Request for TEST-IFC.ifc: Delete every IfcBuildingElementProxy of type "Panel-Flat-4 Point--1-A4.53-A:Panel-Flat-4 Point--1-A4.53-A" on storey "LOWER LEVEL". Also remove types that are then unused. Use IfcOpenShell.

First a look at what the model holds.

```python
import ifcopenshell
import ifcopenshell.util.element

model = ifcopenshell.open("TEST-IFC.ifc")
print(model.schema)
storey = next(s for s in model.by_type("IfcBuildingStorey") if s.Name == "LOWER LEVEL")
proxies = [e for e in ifcopenshell.util.element.get_decomposition(storey) if e.is_a("IfcBuildingElementProxy")]
seen = {}
for e in proxies:
    element_type = ifcopenshell.util.element.get_type(e)
    name = element_type.Name if element_type not in (None, e) else None
    seen[name] = seen.get(name, 0) + 1
for name, count in sorted(seen.items(), key=str):
    print(count, "x", name)
```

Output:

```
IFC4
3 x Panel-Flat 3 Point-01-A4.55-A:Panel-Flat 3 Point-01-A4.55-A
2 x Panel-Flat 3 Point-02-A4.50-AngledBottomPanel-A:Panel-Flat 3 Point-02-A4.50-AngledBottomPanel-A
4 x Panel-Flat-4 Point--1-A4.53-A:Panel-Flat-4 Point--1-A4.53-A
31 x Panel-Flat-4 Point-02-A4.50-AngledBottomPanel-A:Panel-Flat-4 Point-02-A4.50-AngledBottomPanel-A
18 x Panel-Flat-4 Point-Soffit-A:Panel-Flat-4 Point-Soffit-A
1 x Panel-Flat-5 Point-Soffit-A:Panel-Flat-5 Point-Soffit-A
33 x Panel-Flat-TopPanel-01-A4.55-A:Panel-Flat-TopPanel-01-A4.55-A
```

```python
import ifcopenshell
import ifcopenshell.api.root
import ifcopenshell.util.element

model = ifcopenshell.open("TEST-IFC.ifc")

storey = next(s for s in model.by_type("IfcBuildingStorey") if s.Name == "LOWER LEVEL")
proxies = [e for e in ifcopenshell.util.element.get_decomposition(storey) if e.is_a("IfcBuildingElementProxy")]
targets = [e for e in proxies if (t := ifcopenshell.util.element.get_type(e)) not in (None, e) and t.Name == "Panel-Flat-4 Point--1-A4.53-A:Panel-Flat-4 Point--1-A4.53-A"]
types = {ifcopenshell.util.element.get_type(e) for e in targets} - {None, *targets}

for e in targets:
    ifcopenshell.api.root.remove_product(model, product=e)
print(len(targets), "removed")

unused = [t for t in types if not ifcopenshell.util.element.get_types(t)]
for t in unused:
    ifcopenshell.api.root.remove_product(model, product=t)
print(len(unused), "unused types removed")

model.write("TEST-IFC_updated.ifc")
```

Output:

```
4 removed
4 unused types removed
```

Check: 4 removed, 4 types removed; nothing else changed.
